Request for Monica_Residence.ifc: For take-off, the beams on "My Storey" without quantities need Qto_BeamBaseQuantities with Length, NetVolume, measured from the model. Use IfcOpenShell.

First a look at what the model holds.

```python
import ifcopenshell
import ifcopenshell.util.element
import ifcopenshell.util.unit

model = ifcopenshell.open("Monica_Residence.ifc")
print(model.schema)
for unit_type in ("LENGTHUNIT", "AREAUNIT", "VOLUMEUNIT"):
    print(unit_type, ifcopenshell.util.unit.calculate_unit_scale(model, unit_type))
storey = next(s for s in model.by_type("IfcBuildingStorey") if s.Name == "My Storey")
beams = [e for e in ifcopenshell.util.element.get_decomposition(storey) if e.is_a("IfcBeam")]
for e in sorted(beams, key=lambda e: e.id()):
    print(e.id(), e.is_a(), e.Name, list(ifcopenshell.util.element.get_psets(e, qtos_only=True)), sep=" | ")
```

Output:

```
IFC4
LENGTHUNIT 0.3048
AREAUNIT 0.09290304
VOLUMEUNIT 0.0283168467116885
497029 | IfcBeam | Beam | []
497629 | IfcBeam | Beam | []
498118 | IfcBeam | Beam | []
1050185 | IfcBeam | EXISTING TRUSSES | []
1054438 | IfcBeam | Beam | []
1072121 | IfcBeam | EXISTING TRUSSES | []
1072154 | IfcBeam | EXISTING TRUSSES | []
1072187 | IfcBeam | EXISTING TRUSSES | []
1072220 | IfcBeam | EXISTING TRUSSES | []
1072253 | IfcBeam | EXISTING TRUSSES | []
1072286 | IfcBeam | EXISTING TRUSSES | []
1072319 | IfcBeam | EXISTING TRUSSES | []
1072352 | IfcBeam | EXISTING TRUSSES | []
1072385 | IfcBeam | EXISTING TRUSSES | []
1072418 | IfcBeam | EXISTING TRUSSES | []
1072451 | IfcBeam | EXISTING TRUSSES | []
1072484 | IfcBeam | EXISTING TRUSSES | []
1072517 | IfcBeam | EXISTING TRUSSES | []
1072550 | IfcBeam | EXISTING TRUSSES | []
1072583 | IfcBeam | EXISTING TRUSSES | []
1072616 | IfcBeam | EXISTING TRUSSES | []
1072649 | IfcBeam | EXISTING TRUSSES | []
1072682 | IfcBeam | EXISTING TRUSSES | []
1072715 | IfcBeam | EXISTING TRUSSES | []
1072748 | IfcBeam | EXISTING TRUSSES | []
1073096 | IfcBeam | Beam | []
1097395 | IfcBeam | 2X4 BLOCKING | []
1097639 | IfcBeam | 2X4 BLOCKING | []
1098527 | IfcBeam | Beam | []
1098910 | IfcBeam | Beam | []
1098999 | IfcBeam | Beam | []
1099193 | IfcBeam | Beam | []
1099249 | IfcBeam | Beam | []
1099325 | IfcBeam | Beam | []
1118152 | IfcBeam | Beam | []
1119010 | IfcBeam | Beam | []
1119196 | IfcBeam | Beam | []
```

```python
import ifcopenshell
import ifcopenshell.api.pset
import ifcopenshell.geom
import ifcopenshell.util.element
import ifcopenshell.util.shape
import ifcopenshell.util.unit

model = ifcopenshell.open("Monica_Residence.ifc")
unit_scale = ifcopenshell.util.unit.calculate_unit_scale(model)
volume_scale = ifcopenshell.util.unit.calculate_unit_scale(model, "VOLUMEUNIT")
settings = ifcopenshell.geom.settings()

storey = next(s for s in model.by_type("IfcBuildingStorey") if s.Name == "My Storey")
beams = [e for e in ifcopenshell.util.element.get_decomposition(storey) if e.is_a("IfcBeam")]

for e in sorted(beams, key=lambda e: e.id()):
    if ifcopenshell.util.element.get_psets(e, qtos_only=True, should_inherit=False):
        continue
    # Geometry comes back in metres, in the element's own axes.
    shape = ifcopenshell.geom.create_shape(settings, e)
    values = {
        "Length": ifcopenshell.util.shape.get_max_xyz(shape.geometry) / unit_scale,
        "NetVolume": ifcopenshell.util.shape.get_volume(shape.geometry) / volume_scale,
    }
    qto = ifcopenshell.api.pset.add_qto(model, product=e, name="Qto_BeamBaseQuantities")
    ifcopenshell.api.pset.edit_qto(model, qto=qto, properties=values)
    print(e.id(), {k: round(v, 3) for k, v in values.items()})

model.write("Monica_Residence_v2.ifc")
```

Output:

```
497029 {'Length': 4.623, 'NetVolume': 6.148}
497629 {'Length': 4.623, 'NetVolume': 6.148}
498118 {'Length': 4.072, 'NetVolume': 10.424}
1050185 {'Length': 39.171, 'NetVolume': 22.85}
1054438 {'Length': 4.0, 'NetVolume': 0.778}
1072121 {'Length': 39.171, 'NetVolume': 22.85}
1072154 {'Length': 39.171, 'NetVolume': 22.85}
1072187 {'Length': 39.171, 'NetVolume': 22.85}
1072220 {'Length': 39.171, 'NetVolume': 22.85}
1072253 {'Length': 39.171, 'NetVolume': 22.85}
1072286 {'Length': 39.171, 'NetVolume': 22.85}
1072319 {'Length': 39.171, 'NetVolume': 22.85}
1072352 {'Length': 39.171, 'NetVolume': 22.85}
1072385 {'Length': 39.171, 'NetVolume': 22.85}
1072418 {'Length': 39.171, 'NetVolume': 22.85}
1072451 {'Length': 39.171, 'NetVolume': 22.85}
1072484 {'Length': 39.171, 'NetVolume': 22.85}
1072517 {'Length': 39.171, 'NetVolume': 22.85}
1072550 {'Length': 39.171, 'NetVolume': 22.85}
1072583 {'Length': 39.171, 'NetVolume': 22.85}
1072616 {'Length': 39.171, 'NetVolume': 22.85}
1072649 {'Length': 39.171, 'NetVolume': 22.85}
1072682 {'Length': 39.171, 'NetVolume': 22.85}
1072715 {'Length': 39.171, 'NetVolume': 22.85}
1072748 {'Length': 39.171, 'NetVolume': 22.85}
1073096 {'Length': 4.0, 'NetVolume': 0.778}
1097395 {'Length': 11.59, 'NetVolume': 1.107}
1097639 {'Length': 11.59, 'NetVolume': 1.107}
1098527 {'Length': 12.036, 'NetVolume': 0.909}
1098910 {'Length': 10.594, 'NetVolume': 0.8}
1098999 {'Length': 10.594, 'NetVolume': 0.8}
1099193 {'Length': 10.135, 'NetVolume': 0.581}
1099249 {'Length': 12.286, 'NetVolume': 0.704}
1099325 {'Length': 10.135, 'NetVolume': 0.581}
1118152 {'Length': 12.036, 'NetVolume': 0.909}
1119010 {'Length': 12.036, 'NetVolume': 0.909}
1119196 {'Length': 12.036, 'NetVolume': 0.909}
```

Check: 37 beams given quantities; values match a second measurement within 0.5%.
